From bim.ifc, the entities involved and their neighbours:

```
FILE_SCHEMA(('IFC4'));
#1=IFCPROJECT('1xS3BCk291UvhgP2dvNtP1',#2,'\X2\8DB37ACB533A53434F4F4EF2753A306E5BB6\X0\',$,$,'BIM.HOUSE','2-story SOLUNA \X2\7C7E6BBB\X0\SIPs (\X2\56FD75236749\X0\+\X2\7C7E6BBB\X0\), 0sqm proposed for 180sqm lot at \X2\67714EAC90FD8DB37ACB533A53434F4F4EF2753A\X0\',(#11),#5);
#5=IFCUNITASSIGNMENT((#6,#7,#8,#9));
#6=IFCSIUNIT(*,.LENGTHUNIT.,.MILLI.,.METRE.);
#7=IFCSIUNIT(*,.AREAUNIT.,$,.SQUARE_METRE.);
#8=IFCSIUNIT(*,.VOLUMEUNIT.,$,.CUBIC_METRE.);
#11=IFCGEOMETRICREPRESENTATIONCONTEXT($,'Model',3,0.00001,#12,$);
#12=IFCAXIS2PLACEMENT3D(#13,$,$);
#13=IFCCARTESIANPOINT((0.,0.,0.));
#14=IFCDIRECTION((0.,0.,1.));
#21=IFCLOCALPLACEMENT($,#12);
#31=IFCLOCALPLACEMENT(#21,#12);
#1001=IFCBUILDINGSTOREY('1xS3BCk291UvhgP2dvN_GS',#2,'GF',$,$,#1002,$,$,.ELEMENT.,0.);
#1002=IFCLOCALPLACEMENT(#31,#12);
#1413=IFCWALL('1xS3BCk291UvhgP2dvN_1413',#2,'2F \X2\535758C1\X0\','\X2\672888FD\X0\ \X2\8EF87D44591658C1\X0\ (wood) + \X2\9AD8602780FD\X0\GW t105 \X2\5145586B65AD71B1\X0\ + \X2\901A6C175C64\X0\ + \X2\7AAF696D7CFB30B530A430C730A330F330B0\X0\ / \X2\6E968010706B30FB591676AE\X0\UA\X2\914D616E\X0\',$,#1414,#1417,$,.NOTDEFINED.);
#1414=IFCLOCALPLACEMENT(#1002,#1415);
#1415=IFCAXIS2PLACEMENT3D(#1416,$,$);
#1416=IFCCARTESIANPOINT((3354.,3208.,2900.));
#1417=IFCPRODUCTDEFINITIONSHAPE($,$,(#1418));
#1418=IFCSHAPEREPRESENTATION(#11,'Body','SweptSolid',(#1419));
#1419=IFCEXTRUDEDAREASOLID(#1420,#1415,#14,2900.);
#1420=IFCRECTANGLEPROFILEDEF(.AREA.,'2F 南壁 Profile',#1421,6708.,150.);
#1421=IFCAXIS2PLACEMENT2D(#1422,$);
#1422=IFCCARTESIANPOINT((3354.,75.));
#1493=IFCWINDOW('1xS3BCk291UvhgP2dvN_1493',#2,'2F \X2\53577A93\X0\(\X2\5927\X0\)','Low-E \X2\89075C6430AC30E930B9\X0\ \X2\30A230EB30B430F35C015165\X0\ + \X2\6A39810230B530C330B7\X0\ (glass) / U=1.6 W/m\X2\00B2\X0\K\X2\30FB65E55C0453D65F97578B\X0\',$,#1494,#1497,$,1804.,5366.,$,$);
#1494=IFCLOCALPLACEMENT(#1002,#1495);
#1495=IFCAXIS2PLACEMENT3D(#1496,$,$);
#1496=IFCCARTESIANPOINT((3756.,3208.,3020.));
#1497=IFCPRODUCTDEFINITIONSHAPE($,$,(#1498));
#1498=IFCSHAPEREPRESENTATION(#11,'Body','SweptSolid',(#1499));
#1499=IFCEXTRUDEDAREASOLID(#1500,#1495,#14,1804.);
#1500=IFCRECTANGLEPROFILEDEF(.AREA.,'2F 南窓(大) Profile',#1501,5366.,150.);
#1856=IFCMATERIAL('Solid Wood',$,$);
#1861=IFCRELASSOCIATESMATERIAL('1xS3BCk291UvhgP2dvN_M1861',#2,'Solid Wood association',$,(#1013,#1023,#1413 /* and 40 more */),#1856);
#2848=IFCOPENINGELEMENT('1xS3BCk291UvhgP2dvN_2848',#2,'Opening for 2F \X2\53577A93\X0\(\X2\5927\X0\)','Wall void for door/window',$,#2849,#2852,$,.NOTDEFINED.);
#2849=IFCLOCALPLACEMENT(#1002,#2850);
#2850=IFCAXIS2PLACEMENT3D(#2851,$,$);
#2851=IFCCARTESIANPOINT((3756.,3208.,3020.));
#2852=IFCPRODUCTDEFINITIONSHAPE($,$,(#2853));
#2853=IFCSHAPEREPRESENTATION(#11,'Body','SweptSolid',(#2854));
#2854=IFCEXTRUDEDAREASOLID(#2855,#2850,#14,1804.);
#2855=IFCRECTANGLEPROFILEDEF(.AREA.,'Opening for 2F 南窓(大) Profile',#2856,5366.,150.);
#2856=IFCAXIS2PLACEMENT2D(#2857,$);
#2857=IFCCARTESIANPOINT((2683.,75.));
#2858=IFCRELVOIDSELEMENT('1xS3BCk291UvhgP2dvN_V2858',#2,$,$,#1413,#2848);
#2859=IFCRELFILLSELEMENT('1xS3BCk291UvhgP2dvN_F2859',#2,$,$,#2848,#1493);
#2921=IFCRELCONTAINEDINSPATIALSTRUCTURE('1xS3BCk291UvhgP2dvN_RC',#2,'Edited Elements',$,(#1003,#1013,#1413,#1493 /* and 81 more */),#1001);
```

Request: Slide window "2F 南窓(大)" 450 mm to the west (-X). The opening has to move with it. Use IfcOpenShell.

```python
import ifcopenshell
import ifcopenshell.api.geometry
import ifcopenshell.util.placement
import ifcopenshell.util.unit

model = ifcopenshell.open("bim.ifc")
unit_scale = ifcopenshell.util.unit.calculate_unit_scale(model)

window = model.by_id(1493)
opening = window.FillsVoids[0].RelatingOpeningElement
wall = opening.VoidsElements[0].RelatingBuildingElement

wall_matrix = ifcopenshell.util.placement.get_local_placement(wall.ObjectPlacement)
shift = wall_matrix[:3, 0] * -0.45 / unit_scale
before = ifcopenshell.util.placement.get_local_placement(window.ObjectPlacement)[:3, 3].copy()

# The window is not placed relative to its opening, so move both.
for product in (opening, window):
    matrix = ifcopenshell.util.placement.get_local_placement(product.ObjectPlacement)
    matrix[:3, 3] += shift
    ifcopenshell.api.geometry.edit_object_placement(model, product=product, matrix=matrix, is_si=False)

after = ifcopenshell.util.placement.get_local_placement(window.ObjectPlacement)[:3, 3]
print("window moved by", (after - before).round(3) + 0.0)

model.write("bim_updated.ifc")
```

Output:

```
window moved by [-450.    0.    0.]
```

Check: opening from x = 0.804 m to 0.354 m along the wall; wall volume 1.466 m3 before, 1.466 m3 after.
